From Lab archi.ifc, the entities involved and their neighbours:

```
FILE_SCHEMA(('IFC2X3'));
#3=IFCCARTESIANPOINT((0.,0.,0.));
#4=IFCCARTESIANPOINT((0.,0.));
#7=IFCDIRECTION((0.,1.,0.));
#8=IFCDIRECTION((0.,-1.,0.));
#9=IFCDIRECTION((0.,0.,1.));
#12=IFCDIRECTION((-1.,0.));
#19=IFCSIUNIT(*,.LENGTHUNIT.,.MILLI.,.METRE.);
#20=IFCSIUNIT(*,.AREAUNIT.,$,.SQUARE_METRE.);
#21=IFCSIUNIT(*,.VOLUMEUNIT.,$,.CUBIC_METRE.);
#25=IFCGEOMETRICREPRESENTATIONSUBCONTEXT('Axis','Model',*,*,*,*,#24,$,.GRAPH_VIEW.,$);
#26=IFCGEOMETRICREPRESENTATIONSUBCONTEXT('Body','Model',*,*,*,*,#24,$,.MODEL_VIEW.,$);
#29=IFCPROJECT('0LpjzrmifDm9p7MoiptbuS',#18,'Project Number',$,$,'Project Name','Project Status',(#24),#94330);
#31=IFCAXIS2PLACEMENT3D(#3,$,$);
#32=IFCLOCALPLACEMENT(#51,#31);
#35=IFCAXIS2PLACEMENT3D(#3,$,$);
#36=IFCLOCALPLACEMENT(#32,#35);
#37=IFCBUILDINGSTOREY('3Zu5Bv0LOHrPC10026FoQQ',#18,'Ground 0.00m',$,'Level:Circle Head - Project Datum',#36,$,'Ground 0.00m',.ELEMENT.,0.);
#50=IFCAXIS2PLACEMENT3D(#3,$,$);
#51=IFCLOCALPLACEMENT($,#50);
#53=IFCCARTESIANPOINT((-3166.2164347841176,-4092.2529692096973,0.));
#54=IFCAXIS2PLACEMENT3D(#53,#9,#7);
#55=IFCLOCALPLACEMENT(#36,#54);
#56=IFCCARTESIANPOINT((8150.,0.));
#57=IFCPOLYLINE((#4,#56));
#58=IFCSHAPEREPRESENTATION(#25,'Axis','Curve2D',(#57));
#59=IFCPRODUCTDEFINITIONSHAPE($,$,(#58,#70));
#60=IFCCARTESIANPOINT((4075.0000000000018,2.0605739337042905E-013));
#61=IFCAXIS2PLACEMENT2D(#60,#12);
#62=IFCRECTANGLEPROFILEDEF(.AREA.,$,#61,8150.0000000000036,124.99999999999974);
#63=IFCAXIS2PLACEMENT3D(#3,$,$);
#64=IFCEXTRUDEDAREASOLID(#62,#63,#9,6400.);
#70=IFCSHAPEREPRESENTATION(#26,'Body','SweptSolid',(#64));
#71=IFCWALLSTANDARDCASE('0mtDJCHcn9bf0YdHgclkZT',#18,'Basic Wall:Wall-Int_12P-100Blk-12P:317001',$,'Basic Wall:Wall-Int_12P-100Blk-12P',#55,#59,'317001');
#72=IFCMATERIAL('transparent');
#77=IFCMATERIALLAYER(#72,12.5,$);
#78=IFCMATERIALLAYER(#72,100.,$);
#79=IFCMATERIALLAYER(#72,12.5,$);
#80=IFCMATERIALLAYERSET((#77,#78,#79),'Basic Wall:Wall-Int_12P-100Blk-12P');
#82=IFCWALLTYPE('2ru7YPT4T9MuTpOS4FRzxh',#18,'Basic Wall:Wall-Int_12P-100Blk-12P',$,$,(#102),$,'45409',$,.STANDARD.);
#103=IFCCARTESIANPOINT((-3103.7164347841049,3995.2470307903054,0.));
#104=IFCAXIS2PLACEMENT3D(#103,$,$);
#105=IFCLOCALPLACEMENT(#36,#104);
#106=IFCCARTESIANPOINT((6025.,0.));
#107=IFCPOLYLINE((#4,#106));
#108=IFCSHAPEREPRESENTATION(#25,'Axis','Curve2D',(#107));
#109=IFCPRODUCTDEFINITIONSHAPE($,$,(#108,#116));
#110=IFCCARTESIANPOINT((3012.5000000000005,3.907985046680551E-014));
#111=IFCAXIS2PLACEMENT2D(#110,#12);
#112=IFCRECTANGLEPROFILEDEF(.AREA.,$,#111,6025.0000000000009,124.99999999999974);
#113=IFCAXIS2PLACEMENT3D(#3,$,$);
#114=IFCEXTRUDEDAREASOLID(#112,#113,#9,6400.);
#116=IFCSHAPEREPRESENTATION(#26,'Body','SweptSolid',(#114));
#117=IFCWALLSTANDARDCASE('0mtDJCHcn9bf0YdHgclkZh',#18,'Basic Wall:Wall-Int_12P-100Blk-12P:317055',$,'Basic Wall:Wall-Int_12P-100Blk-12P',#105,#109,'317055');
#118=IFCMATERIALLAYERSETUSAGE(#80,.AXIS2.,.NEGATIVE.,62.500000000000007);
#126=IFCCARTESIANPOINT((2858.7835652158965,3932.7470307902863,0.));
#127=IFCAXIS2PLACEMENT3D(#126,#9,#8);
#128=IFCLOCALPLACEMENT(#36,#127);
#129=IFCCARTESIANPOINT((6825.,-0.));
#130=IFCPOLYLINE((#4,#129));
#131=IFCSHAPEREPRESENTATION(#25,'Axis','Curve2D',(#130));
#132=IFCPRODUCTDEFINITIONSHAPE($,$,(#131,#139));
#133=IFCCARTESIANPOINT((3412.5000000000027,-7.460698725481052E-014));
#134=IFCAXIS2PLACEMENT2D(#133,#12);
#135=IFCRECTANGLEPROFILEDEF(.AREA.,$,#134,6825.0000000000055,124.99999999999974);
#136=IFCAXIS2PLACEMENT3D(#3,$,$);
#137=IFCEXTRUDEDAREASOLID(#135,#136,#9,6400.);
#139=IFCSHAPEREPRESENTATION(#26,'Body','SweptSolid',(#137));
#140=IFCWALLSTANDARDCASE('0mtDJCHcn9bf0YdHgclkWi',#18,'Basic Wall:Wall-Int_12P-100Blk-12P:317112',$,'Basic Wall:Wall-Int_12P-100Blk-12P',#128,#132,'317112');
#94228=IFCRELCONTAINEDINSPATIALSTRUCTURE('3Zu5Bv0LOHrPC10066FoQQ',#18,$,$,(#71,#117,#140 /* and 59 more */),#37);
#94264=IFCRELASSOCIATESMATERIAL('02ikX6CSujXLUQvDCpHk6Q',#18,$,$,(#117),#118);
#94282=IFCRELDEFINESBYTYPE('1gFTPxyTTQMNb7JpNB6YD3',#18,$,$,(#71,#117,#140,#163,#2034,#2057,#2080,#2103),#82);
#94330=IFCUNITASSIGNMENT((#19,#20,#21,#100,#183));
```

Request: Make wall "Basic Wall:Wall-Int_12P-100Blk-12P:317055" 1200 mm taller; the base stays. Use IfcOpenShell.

```python
import ifcopenshell
import ifcopenshell.geom
import ifcopenshell.util.representation
import ifcopenshell.util.shape

model = ifcopenshell.open("Lab archi.ifc")
settings = ifcopenshell.geom.settings()


def volume(element):
    """Net volume in cubic metres, openings subtracted."""
    shape = ifcopenshell.geom.create_shape(settings, element)
    return ifcopenshell.util.shape.get_volume(shape.geometry)


wall = model.by_id(117)
before = volume(wall)

body = ifcopenshell.util.representation.get_representation(wall, "Model", "Body")
solid = body.Items[0]
old_height = solid.Depth
solid.Depth += 1200.0
after = volume(wall)

print(f"height {old_height:g} -> {solid.Depth:g}, volume {before:.3f} -> {after:.3f} m3")

model.write("Lab archi_v2.ifc")
```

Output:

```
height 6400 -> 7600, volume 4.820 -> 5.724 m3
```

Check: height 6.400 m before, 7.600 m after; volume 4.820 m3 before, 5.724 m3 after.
